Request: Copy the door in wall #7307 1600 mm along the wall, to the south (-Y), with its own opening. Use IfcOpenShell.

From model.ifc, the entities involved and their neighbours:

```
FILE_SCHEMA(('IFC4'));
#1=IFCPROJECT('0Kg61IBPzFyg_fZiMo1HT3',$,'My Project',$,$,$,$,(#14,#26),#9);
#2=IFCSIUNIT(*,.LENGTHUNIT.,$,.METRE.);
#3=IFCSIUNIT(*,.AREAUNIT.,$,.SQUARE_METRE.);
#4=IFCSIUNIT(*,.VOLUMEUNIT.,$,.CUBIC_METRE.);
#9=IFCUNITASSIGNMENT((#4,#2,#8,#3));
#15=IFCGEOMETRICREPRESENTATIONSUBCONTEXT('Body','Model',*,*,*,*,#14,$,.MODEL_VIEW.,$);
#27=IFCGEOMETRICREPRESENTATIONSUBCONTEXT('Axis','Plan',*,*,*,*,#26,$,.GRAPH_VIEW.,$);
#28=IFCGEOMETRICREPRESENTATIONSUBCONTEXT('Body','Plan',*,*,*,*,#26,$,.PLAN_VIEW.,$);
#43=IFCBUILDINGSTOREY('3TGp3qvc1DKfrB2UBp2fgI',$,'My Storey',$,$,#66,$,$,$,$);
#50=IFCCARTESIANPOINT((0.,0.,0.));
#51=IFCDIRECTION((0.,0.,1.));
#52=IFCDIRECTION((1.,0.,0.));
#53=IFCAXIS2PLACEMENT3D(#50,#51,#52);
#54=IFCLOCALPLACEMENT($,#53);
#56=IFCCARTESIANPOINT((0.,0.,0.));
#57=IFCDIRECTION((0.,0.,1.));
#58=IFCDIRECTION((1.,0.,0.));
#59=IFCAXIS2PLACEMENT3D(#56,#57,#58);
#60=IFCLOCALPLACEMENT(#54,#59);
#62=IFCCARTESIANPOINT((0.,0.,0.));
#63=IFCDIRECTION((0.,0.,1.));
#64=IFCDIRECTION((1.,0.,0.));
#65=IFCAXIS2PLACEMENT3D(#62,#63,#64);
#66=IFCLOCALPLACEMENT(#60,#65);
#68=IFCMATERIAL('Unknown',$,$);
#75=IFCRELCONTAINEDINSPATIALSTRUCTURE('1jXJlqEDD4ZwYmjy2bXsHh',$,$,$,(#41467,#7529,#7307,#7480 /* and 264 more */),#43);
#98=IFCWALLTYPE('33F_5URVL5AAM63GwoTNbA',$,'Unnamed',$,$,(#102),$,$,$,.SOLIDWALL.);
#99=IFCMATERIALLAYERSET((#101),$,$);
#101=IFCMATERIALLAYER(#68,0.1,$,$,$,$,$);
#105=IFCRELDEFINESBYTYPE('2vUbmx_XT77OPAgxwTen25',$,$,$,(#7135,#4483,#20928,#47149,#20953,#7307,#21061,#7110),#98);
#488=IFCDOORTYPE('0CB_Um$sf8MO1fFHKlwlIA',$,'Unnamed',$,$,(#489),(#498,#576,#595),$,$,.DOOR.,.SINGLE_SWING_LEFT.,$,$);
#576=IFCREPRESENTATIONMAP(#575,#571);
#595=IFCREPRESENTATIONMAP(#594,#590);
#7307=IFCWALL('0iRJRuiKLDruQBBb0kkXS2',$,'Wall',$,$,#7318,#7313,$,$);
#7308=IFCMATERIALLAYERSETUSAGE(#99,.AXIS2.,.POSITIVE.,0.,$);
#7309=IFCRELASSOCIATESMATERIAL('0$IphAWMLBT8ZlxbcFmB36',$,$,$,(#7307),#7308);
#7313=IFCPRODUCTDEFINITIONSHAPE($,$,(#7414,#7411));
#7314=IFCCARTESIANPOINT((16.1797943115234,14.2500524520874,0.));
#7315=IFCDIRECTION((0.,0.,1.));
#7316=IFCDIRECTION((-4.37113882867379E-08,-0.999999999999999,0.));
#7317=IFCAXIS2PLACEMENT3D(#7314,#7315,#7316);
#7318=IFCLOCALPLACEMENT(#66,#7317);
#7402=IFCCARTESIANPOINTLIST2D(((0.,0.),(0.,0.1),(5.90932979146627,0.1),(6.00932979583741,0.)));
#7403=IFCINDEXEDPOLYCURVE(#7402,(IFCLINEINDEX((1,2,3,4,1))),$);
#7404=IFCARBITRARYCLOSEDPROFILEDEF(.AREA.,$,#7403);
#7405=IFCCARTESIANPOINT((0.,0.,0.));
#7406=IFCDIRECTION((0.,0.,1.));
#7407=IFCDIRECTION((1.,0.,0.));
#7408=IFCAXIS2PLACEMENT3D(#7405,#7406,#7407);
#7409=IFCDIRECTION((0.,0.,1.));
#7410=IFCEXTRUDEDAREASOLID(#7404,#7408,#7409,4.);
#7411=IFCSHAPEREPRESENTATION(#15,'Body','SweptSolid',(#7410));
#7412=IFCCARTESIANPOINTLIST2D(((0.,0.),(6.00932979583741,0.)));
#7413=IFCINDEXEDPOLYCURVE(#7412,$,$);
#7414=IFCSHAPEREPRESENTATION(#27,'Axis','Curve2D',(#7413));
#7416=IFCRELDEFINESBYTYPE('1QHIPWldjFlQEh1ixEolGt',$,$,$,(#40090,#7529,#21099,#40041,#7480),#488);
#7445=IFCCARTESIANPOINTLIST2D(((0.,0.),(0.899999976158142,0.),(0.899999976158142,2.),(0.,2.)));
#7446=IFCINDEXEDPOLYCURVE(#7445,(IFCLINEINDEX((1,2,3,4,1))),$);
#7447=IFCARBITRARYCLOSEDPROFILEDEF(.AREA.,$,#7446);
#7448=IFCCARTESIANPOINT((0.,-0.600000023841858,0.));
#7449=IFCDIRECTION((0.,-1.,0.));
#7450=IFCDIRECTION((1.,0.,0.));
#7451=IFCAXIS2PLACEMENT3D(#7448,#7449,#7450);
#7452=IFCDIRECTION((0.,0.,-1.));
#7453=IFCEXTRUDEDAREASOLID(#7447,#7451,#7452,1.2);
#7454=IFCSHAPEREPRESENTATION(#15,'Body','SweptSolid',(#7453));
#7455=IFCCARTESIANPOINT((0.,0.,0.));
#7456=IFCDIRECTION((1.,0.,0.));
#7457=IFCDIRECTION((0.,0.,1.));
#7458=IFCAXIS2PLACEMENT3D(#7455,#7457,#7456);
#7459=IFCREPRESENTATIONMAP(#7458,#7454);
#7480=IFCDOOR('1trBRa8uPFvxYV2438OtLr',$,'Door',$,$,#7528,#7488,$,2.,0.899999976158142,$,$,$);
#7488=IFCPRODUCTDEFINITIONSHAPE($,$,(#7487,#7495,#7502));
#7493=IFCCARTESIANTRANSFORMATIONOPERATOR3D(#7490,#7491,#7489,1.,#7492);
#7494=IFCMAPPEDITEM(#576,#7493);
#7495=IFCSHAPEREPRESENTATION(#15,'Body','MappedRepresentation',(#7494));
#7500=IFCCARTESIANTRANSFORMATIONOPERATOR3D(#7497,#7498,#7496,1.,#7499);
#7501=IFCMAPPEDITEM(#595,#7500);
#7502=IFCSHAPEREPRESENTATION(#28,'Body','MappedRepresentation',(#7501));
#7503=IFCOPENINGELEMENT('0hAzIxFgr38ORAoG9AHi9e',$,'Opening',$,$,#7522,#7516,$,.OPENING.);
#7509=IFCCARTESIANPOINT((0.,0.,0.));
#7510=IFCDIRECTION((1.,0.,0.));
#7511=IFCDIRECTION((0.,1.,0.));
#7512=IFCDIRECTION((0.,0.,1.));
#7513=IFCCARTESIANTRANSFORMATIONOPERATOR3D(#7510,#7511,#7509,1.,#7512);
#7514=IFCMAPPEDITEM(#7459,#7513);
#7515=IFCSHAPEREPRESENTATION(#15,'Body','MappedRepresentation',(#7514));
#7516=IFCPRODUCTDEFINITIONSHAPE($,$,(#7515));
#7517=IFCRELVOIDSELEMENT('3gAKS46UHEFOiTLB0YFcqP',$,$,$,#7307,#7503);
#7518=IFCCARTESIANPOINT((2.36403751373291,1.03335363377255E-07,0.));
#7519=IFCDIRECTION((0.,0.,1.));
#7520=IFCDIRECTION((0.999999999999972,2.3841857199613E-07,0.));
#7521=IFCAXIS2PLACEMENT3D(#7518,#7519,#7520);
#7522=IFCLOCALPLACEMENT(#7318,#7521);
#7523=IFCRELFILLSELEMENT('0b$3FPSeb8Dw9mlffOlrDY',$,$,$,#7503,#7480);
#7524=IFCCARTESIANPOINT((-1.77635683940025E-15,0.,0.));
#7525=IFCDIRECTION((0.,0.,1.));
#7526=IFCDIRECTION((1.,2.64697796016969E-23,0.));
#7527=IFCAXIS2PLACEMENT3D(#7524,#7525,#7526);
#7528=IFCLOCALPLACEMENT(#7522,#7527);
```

```python
import ifcopenshell
import ifcopenshell.api.feature
import ifcopenshell.api.geometry
import ifcopenshell.api.root
import ifcopenshell.geom
import ifcopenshell.util.element
import ifcopenshell.util.placement
import ifcopenshell.util.shape
import ifcopenshell.util.unit

model = ifcopenshell.open("model.ifc")
unit_scale = ifcopenshell.util.unit.calculate_unit_scale(model)
settings = ifcopenshell.geom.settings()


def volume(element):
    """Net volume in cubic metres, openings subtracted."""
    shape = ifcopenshell.geom.create_shape(settings, element)
    return ifcopenshell.util.shape.get_volume(shape.geometry)


door = model.by_guid("1trBRa8uPFvxYV2438OtLr")
opening = door.FillsVoids[0].RelatingOpeningElement
wall = opening.VoidsElements[0].RelatingBuildingElement
before = volume(wall)
shift = ifcopenshell.util.placement.get_local_placement(wall.ObjectPlacement)[:3, 0] * 1.6 / unit_scale

# copy_class copies the void relationship, type, container and properties, but no geometry.
new_opening = ifcopenshell.api.root.copy_class(model, product=opening)
new_opening.Representation = ifcopenshell.util.element.copy_deep(
    model, opening.Representation, exclude=["IfcGeometricRepresentationContext", "IfcRepresentationMap"]
)
new_door = ifcopenshell.api.root.copy_class(model, product=door)
new_door.Representation = ifcopenshell.util.element.copy_deep(
    model, door.Representation, exclude=["IfcGeometricRepresentationContext", "IfcRepresentationMap"]
)
ifcopenshell.api.feature.add_filling(model, opening=new_opening, element=new_door)

for old, new in ((opening, new_opening), (door, new_door)):
    matrix = ifcopenshell.util.placement.get_local_placement(old.ObjectPlacement)
    matrix[:3, 3] += shift
    ifcopenshell.api.geometry.edit_object_placement(model, product=new, matrix=matrix, is_si=False)

after = volume(wall)

print(f"wall volume {before:.3f} -> {after:.3f} m3")

model.write("model_v2.ifc")
```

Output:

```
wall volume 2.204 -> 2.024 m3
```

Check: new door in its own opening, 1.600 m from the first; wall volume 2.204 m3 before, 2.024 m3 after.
